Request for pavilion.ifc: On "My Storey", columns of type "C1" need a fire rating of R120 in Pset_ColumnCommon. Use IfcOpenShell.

First a look at what the model holds.

```python
import ifcopenshell
import ifcopenshell.util.element

model = ifcopenshell.open("pavilion.ifc")
print(model.schema)
storey = next(s for s in model.by_type("IfcBuildingStorey") if s.Name == "My Storey")
columns = [e for e in ifcopenshell.util.element.get_decomposition(storey) if e.is_a("IfcColumn")]
seen = {}
for e in columns:
    element_type = ifcopenshell.util.element.get_type(e)
    key = (element_type.Name if element_type != e and element_type else None, ifcopenshell.util.element.get_pset(e, "Pset_ColumnCommon", "FireRating"))
    seen[key] = seen.get(key, 0) + 1
for (name, value), count in sorted(seen.items(), key=str):
    print(count, "x", name, "|", value)
```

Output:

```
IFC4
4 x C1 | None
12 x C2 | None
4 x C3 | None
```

```python
import ifcopenshell
import ifcopenshell.api.pset
import ifcopenshell.util.element

model = ifcopenshell.open("pavilion.ifc")

storey = next(s for s in model.by_type("IfcBuildingStorey") if s.Name == "My Storey")
columns = [e for e in ifcopenshell.util.element.get_decomposition(storey) if e.is_a("IfcColumn")]

count = 0
for e in columns:
    element_type = ifcopenshell.util.element.get_type(e)
    if element_type in (None, e) or element_type.Name != "C1":
        continue
    # add_pset returns the element's existing set when there is one.
    pset = ifcopenshell.api.pset.add_pset(model, product=e, name="Pset_ColumnCommon")
    ifcopenshell.api.pset.edit_pset(model, pset=pset, properties={"FireRating": "R120"})
    count += 1

print(count, "columns updated")

model.write("pavilion_edited.ifc")
```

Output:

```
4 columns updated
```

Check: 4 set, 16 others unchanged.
